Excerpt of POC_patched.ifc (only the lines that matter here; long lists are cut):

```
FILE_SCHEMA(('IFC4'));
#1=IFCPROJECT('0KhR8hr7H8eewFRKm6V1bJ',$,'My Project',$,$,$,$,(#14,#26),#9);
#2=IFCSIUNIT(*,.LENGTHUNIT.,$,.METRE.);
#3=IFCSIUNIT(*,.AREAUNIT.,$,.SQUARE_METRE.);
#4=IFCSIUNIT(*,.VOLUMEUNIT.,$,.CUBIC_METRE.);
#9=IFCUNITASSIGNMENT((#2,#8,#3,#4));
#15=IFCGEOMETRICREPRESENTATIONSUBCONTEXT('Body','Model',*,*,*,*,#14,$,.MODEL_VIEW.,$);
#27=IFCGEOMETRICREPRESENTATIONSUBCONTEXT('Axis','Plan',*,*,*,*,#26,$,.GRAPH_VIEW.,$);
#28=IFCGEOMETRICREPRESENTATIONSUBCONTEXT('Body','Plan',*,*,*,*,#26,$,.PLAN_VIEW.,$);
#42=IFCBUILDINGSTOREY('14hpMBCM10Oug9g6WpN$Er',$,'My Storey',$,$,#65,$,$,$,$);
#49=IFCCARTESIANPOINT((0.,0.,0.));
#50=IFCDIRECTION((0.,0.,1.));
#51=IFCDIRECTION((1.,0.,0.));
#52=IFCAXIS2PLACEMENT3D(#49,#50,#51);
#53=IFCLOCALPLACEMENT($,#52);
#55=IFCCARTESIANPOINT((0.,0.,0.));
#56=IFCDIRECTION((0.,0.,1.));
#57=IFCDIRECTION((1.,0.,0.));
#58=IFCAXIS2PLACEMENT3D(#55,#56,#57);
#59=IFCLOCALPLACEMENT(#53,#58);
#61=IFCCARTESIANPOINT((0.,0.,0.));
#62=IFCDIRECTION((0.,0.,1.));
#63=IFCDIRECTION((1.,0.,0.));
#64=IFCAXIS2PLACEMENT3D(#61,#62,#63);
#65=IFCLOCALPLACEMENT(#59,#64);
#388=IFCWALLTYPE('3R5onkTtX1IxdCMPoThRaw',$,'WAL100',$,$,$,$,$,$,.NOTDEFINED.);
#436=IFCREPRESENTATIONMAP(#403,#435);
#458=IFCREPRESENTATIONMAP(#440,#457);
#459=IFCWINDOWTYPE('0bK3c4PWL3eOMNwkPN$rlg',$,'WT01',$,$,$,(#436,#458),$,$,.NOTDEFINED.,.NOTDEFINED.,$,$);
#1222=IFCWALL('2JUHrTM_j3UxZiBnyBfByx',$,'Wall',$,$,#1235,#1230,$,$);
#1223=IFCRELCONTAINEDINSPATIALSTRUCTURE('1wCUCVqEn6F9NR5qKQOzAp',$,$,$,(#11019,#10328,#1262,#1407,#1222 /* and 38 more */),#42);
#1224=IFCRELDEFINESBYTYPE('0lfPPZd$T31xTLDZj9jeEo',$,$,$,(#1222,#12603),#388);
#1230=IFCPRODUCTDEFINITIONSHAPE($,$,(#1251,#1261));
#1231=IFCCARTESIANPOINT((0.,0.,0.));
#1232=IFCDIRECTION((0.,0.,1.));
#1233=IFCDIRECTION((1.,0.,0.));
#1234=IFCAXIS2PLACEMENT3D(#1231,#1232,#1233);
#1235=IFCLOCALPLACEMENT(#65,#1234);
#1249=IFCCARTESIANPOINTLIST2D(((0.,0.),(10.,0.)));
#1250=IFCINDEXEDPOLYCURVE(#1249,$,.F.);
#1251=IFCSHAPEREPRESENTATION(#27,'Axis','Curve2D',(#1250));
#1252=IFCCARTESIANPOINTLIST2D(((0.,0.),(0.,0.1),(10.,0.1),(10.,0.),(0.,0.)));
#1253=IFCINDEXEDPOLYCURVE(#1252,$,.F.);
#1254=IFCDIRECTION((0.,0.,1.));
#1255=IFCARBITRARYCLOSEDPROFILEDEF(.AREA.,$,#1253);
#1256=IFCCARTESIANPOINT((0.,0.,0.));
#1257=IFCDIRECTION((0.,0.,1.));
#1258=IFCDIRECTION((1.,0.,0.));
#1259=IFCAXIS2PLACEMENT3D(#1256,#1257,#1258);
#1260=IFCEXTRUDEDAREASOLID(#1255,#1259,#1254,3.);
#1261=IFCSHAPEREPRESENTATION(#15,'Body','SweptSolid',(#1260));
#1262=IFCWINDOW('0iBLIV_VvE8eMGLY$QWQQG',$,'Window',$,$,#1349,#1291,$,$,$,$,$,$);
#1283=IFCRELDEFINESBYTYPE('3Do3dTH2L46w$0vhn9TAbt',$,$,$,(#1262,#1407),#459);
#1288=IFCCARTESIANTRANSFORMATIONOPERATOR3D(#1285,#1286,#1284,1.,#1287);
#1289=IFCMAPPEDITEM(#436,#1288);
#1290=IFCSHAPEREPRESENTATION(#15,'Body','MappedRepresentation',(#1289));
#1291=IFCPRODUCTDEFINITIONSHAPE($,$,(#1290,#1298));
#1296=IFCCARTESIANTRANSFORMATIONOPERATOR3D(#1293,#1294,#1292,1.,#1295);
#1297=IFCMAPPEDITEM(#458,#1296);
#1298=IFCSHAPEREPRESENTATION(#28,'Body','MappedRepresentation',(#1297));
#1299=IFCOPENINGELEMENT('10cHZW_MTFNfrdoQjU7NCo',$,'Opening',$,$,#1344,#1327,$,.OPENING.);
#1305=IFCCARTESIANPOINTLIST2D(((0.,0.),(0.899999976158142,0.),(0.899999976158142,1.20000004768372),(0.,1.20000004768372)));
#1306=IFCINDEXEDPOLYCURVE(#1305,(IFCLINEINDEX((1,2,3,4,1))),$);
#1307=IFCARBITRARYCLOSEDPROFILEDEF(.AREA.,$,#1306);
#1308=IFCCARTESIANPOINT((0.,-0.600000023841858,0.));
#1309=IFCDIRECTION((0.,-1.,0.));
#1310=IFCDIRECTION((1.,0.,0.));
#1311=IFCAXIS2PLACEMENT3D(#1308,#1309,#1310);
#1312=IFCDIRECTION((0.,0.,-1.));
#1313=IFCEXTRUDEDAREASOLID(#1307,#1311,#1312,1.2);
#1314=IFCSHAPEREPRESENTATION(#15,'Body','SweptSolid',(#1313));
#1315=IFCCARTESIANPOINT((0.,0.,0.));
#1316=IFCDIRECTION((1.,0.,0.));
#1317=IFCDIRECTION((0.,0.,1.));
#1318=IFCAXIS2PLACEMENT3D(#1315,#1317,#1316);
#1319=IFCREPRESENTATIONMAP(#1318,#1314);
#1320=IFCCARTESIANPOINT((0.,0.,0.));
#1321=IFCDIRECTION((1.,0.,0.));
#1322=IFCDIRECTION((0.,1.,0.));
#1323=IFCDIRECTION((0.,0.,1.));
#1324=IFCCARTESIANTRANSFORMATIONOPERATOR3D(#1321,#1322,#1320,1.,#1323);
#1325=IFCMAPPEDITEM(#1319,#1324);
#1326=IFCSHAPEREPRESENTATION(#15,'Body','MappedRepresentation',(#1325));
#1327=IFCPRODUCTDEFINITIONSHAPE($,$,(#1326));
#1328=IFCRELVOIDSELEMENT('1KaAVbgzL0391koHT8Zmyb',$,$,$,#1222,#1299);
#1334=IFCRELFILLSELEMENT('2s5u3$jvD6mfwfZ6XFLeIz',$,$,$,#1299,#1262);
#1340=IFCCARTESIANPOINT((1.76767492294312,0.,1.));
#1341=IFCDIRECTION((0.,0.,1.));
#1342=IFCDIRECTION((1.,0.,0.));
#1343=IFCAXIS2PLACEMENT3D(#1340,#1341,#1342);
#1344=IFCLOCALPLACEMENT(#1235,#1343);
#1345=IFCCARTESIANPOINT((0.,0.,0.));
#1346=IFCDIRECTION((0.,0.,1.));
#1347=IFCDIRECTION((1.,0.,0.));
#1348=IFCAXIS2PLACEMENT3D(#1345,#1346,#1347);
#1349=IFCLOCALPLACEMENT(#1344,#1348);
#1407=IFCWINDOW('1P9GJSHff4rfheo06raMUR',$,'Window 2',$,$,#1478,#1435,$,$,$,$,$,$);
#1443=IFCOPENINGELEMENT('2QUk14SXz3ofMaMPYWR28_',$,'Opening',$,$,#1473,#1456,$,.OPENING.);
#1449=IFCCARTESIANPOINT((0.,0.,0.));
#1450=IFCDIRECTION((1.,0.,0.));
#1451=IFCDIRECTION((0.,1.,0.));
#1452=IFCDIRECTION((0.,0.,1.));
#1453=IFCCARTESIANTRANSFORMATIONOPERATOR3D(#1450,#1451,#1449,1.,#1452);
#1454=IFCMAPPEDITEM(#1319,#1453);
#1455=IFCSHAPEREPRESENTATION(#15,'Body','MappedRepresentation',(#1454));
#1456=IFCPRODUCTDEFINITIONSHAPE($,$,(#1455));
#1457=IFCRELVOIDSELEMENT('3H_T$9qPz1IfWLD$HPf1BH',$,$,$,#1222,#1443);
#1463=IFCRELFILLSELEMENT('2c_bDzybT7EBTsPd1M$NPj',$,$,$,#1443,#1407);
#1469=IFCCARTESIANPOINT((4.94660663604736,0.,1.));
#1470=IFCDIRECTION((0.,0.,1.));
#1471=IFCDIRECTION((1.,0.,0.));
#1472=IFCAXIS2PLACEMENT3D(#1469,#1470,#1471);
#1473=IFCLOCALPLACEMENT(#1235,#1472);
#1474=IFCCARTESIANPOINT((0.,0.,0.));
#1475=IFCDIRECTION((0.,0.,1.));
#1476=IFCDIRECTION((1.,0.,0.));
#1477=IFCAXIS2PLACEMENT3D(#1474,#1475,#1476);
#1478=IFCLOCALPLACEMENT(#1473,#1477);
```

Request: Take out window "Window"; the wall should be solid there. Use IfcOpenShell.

```python
import ifcopenshell
import ifcopenshell.api.feature
import ifcopenshell.api.root
import ifcopenshell.geom
import ifcopenshell.util.shape

model = ifcopenshell.open("POC_patched.ifc")
settings = ifcopenshell.geom.settings()


def volume(element):
    """Net volume in cubic metres, openings subtracted."""
    shape = ifcopenshell.geom.create_shape(settings, element)
    return ifcopenshell.util.shape.get_volume(shape.geometry)


window = model.by_id(1262)
opening = window.FillsVoids[0].RelatingOpeningElement
wall = opening.VoidsElements[0].RelatingBuildingElement
before = volume(wall)

ifcopenshell.api.root.remove_product(model, product=window)
ifcopenshell.api.feature.remove_feature(model, feature=opening)

after = volume(wall)

print(f"wall volume {before:.3f} -> {after:.3f} m3")

model.write("POC_patched_rev.ifc")
```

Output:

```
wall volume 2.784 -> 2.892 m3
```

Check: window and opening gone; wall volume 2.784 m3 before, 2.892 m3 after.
